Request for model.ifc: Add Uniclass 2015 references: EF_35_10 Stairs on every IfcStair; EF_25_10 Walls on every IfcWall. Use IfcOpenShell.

First a look at what the model holds.

```python
import ifcopenshell

model = ifcopenshell.open("model.ifc")
print(model.schema)
print("classifications:", [c.Name for c in model.by_type("IfcClassification")])
for ifc_class in ("IfcDoor", "IfcRoof", "IfcStair", "IfcWall", "IfcWindow"):
    print(ifc_class, len(model.by_type(ifc_class)))
```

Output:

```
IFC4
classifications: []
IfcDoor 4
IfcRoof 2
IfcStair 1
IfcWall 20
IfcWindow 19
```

```python
import ifcopenshell
import ifcopenshell.api.classification

model = ifcopenshell.open("model.ifc")

system = ifcopenshell.api.classification.add_classification(model, classification="Uniclass 2015")

codes = {
    "IfcStair": ("EF_35_10", "Stairs"),
    "IfcWall": ("EF_25_10", "Walls"),
}
for ifc_class, (code, name) in codes.items():
    products = model.by_type(ifc_class)
    ifcopenshell.api.classification.add_reference(
        model, products=products, classification=system, identification=code, name=name
    )
    print(code, len(products))

model.write("model-out.ifc")
```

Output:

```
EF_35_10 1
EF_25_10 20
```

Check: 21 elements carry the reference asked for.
